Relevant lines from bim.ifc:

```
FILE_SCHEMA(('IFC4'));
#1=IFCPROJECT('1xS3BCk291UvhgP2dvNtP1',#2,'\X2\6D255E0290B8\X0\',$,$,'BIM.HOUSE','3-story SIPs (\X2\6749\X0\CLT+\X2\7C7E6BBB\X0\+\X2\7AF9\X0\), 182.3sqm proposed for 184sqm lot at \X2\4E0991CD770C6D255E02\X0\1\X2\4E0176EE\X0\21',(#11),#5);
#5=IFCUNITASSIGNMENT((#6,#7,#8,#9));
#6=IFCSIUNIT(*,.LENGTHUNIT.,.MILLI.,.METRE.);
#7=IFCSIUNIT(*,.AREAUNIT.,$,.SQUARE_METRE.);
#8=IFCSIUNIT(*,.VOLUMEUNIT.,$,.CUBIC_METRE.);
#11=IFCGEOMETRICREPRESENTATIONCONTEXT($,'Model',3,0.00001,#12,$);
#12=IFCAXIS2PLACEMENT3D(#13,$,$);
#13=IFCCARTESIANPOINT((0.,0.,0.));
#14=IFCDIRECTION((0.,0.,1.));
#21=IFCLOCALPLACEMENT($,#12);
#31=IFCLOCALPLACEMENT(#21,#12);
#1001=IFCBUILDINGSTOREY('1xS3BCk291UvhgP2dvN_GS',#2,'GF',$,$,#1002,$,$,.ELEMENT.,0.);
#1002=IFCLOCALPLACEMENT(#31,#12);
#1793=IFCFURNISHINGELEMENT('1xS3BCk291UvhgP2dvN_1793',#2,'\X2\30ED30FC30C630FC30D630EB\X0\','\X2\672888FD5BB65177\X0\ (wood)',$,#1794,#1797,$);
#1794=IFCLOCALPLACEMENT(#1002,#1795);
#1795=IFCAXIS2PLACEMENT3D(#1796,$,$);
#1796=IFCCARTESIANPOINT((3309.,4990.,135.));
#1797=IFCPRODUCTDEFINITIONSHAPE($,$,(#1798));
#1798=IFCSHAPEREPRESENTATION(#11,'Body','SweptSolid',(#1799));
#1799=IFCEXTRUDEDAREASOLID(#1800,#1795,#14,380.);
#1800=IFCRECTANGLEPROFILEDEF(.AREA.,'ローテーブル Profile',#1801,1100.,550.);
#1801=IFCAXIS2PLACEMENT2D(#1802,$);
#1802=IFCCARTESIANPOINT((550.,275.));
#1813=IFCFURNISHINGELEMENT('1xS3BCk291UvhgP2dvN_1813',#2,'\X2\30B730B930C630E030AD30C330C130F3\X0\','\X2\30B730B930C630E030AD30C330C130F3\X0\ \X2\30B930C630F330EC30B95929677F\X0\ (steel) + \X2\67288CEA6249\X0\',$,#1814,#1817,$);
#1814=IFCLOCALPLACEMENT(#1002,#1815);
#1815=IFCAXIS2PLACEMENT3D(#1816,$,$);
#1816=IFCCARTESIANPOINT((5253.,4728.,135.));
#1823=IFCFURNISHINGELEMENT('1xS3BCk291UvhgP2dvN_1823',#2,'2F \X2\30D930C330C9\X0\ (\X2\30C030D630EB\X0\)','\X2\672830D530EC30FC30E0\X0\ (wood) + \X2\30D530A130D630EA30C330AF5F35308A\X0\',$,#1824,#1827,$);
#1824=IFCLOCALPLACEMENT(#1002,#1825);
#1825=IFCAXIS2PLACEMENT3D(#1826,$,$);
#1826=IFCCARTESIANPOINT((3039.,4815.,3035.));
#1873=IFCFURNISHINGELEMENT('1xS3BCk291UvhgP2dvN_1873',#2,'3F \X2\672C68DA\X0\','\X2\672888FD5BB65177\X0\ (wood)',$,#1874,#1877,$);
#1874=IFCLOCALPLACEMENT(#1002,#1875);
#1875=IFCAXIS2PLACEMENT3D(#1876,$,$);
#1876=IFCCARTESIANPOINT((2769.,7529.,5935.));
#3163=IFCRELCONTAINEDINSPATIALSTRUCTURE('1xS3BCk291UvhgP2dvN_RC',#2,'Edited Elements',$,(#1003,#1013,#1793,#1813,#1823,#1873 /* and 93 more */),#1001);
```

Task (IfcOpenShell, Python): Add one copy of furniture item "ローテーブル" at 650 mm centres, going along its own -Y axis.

```python
import ifcopenshell
import ifcopenshell.api.geometry
import ifcopenshell.api.root
import ifcopenshell.util.element
import ifcopenshell.util.placement

model = ifcopenshell.open("bim.ifc")


def reuse_history(source, copy):
    """copy_class also copies each property set's owner history, people and application; keep the originals."""
    for rel in copy.IsDefinedBy:
        if rel.is_a("IfcRelDefinesByProperties") and (history := rel.RelatingPropertyDefinition.OwnerHistory):
            rel.RelatingPropertyDefinition.OwnerHistory = source.OwnerHistory
            ifcopenshell.util.element.remove_deep2(model, history)


source = model.by_id(1793)
base = ifcopenshell.util.placement.get_local_placement(source.ObjectPlacement)
step = -base[:3, 1] * 650.0

for i in range(1, 2):
    copy = ifcopenshell.api.root.copy_class(model, product=source)
    copy.Representation = ifcopenshell.util.element.copy_deep(
        model, source.Representation, exclude=["IfcGeometricRepresentationContext", "IfcRepresentationMap"]
    )
    reuse_history(source, copy)
    matrix = base.copy()
    matrix[:3, 3] += i * step
    print("added at", matrix[:3, 3].round(3) + 0.0)
    ifcopenshell.api.geometry.edit_object_placement(model, product=copy, matrix=matrix, is_si=False)

model.write("bim_rev.ifc")
```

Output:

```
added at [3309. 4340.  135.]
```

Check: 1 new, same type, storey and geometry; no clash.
